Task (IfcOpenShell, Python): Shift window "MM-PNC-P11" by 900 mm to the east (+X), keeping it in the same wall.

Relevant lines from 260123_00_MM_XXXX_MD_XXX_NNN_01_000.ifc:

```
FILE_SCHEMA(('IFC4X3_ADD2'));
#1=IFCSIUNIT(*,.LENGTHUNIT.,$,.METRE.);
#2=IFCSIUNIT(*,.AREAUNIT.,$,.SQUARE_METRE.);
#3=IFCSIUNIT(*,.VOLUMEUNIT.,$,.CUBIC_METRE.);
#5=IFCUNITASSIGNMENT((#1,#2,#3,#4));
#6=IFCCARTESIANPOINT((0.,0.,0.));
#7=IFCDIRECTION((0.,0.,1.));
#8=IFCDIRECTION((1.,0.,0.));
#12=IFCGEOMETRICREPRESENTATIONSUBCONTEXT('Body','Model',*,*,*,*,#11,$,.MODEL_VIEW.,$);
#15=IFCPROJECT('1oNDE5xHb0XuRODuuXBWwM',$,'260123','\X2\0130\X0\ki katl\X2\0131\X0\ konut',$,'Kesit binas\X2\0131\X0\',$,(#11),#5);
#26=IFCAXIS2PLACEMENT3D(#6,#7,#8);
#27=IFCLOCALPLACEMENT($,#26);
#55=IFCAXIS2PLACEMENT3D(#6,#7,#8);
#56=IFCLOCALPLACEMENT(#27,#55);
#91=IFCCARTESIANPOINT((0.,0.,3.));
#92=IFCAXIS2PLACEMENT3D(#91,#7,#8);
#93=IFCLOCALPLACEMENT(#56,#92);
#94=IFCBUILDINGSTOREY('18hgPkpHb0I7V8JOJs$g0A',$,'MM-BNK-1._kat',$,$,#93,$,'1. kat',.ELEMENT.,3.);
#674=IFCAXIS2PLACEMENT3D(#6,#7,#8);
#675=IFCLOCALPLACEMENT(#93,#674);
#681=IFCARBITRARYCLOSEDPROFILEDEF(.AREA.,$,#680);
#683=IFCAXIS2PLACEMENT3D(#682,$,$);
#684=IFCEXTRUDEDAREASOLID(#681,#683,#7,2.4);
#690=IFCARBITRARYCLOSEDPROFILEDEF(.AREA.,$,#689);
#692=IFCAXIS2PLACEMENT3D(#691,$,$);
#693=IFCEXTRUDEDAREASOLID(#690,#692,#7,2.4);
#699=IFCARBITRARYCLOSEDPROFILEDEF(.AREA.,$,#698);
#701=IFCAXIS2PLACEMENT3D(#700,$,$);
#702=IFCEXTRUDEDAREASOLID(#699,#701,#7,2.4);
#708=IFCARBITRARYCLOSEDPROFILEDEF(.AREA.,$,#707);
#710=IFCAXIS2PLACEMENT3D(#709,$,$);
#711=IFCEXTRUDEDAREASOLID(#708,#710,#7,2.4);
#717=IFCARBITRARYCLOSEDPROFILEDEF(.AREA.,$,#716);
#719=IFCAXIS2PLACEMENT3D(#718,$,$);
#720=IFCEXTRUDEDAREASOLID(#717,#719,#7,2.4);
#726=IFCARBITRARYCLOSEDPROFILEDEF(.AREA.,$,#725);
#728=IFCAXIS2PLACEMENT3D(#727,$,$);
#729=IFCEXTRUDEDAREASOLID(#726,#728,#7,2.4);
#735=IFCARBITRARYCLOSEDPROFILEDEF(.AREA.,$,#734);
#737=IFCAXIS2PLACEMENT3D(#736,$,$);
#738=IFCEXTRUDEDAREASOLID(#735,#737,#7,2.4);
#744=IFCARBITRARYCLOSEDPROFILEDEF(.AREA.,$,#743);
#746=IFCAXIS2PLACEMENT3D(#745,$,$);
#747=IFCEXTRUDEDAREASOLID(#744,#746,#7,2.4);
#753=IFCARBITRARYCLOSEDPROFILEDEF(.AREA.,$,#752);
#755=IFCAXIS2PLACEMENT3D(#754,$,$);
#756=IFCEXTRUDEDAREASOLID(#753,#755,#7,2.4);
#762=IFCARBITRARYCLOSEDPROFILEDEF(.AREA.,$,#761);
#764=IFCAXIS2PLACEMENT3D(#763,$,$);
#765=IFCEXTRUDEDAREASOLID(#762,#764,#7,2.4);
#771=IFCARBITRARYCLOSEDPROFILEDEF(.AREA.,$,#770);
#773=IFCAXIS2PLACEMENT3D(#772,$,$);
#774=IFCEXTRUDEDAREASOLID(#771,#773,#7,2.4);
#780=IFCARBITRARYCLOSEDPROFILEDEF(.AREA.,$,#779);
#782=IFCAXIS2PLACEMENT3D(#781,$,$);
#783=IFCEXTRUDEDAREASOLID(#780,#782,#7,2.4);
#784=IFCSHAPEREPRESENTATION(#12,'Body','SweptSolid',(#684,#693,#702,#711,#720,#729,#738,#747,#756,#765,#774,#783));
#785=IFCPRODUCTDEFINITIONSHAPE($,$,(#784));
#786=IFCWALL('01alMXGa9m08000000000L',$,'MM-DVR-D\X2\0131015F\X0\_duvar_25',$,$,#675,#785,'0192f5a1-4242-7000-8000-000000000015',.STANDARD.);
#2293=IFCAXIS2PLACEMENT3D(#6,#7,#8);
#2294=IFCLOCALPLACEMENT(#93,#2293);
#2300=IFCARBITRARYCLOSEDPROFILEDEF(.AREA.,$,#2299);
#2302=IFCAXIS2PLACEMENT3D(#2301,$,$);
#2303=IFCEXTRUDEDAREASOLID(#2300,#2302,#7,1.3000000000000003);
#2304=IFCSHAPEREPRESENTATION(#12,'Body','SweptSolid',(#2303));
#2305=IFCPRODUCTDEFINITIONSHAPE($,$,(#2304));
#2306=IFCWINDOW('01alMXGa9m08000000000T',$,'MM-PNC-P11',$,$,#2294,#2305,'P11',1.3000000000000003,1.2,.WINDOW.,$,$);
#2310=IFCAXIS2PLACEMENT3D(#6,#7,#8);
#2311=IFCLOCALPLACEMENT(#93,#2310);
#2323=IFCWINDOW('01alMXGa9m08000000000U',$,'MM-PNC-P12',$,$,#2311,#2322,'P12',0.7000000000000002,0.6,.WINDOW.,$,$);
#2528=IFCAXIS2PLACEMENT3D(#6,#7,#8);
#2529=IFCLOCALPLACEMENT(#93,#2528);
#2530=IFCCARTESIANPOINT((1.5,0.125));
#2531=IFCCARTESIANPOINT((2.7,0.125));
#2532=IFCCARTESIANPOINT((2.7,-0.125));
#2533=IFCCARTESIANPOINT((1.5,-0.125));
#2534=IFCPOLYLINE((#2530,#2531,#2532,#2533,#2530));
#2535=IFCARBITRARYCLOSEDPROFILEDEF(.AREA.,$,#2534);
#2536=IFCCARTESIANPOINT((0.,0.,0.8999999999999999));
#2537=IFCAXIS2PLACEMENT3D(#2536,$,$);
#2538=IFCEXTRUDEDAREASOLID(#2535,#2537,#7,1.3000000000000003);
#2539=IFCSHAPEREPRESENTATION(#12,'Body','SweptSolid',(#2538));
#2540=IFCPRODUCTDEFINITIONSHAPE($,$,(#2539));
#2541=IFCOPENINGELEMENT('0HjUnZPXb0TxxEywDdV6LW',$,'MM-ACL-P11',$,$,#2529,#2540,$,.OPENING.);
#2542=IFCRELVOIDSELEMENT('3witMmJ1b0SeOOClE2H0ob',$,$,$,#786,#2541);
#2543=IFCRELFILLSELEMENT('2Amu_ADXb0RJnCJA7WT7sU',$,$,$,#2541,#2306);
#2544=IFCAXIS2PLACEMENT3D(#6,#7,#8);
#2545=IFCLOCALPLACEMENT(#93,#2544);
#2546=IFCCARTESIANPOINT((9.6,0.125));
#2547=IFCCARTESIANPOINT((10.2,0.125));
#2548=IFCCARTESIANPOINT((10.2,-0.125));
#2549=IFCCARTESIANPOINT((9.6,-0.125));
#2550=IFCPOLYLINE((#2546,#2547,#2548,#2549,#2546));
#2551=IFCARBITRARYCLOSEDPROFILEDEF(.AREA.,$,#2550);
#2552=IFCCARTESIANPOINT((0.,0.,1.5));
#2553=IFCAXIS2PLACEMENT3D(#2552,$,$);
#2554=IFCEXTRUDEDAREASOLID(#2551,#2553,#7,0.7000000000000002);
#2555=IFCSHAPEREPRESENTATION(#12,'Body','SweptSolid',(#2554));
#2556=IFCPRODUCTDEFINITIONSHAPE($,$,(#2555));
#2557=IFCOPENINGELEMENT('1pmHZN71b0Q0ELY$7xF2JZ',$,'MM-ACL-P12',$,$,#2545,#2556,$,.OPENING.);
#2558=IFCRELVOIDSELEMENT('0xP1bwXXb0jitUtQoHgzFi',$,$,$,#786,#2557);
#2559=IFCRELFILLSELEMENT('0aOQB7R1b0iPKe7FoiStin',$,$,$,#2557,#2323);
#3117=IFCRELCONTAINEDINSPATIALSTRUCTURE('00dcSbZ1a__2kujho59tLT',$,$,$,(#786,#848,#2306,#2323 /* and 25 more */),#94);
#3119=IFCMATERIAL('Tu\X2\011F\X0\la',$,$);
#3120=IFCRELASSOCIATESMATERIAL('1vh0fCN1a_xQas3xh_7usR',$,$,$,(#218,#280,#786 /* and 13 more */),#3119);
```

```python
import ifcopenshell
import ifcopenshell.api.geometry
import ifcopenshell.util.placement
import ifcopenshell.util.unit

model = ifcopenshell.open("260123_00_MM_XXXX_MD_XXX_NNN_01_000.ifc")
unit_scale = ifcopenshell.util.unit.calculate_unit_scale(model)

window = model.by_id(2306)
opening = window.FillsVoids[0].RelatingOpeningElement
wall = opening.VoidsElements[0].RelatingBuildingElement

wall_matrix = ifcopenshell.util.placement.get_local_placement(wall.ObjectPlacement)
shift = wall_matrix[:3, 0] * 0.9 / unit_scale
before = ifcopenshell.util.placement.get_local_placement(window.ObjectPlacement)[:3, 3].copy()

# The window is not placed relative to its opening, so move both.
for product in (opening, window):
    matrix = ifcopenshell.util.placement.get_local_placement(product.ObjectPlacement)
    matrix[:3, 3] += shift
    ifcopenshell.api.geometry.edit_object_placement(model, product=product, matrix=matrix, is_si=False)

after = ifcopenshell.util.placement.get_local_placement(window.ObjectPlacement)[:3, 3]
print("window moved by", (after - before).round(3) + 0.0)

model.write("260123_00_MM_XXXX_MD_XXX_NNN_01_000_updated.ifc")
```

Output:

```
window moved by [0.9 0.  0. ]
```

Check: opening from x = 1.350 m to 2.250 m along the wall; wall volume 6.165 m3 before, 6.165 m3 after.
